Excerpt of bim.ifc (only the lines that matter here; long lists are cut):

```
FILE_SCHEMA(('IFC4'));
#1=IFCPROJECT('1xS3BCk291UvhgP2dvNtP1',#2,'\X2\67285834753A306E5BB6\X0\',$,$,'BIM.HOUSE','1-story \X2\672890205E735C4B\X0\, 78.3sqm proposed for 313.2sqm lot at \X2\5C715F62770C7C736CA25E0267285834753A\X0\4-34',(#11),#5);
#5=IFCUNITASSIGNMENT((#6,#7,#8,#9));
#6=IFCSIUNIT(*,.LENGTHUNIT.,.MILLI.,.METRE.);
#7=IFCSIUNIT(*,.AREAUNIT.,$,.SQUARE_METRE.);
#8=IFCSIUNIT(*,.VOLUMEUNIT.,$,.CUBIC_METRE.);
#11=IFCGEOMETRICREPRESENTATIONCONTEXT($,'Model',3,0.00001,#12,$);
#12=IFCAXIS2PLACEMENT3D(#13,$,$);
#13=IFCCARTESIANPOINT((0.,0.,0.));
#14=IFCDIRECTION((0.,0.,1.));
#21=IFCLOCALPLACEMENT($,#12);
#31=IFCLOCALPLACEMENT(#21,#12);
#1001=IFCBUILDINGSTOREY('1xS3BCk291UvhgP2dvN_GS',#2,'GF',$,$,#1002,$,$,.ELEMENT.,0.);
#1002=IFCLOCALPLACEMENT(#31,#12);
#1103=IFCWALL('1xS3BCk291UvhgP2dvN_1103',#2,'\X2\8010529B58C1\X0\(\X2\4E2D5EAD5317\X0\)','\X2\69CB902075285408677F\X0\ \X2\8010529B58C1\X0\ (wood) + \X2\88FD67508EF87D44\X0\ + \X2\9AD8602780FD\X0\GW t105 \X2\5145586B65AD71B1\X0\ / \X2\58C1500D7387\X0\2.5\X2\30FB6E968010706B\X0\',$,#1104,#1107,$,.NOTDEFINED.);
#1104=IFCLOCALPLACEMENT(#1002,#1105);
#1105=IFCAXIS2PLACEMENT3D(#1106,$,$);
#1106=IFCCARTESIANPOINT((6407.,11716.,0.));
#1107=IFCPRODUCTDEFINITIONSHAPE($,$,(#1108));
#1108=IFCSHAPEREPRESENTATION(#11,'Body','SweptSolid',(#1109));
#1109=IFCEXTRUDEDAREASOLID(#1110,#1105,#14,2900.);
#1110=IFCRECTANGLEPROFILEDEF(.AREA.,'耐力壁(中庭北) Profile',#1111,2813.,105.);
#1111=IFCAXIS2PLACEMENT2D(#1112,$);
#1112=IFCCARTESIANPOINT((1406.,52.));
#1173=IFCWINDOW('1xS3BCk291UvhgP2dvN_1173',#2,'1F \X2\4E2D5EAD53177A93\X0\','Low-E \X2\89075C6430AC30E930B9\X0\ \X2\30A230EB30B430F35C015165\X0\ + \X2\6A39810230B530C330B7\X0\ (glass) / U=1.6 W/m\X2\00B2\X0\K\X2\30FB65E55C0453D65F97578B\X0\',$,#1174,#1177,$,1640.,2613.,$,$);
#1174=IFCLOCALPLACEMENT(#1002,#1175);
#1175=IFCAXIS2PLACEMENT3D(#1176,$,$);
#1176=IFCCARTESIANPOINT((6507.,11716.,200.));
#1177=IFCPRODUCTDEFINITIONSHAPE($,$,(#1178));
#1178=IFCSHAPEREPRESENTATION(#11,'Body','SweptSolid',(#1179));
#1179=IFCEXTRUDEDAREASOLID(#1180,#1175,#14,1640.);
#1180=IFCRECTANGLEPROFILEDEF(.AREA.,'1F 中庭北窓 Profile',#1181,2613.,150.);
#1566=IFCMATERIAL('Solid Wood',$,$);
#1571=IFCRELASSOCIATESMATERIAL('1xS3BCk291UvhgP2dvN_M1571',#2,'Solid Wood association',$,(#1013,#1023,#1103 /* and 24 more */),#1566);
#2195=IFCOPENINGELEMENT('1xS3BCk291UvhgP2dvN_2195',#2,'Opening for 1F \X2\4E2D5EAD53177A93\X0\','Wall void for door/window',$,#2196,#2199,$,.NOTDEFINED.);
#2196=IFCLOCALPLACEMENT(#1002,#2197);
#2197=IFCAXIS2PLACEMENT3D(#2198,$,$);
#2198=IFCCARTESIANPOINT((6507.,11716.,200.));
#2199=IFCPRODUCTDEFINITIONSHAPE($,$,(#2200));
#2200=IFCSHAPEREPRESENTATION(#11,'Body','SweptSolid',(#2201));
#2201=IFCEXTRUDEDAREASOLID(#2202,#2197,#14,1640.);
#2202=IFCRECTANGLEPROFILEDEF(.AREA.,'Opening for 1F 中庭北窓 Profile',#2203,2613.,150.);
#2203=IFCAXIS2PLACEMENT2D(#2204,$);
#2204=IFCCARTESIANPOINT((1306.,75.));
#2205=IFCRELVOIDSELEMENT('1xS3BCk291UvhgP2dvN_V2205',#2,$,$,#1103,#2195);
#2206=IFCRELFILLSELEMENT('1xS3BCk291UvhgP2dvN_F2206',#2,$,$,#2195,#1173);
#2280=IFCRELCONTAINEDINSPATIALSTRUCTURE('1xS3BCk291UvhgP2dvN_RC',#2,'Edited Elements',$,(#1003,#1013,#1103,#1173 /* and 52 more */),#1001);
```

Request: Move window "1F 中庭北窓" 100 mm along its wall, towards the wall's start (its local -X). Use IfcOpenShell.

```python
import ifcopenshell
import ifcopenshell.api.geometry
import ifcopenshell.util.placement

model = ifcopenshell.open("bim.ifc")

window = model.by_guid("1xS3BCk291UvhgP2dvN_1173")
opening = window.FillsVoids[0].RelatingOpeningElement
wall = opening.VoidsElements[0].RelatingBuildingElement

wall_matrix = ifcopenshell.util.placement.get_local_placement(wall.ObjectPlacement)
shift = wall_matrix[:3, 0] * -100.0
before = ifcopenshell.util.placement.get_local_placement(window.ObjectPlacement)[:3, 3].copy()

# The window is not placed relative to its opening, so move both.
for product in (opening, window):
    matrix = ifcopenshell.util.placement.get_local_placement(product.ObjectPlacement)
    matrix[:3, 3] += shift
    ifcopenshell.api.geometry.edit_object_placement(model, product=product, matrix=matrix, is_si=False)

after = ifcopenshell.util.placement.get_local_placement(window.ObjectPlacement)[:3, 3]
print("window moved by", (after - before).round(3) + 0.0)

model.write("bim-out.ifc")
```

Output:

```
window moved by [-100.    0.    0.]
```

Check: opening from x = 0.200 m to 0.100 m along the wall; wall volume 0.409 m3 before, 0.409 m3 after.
